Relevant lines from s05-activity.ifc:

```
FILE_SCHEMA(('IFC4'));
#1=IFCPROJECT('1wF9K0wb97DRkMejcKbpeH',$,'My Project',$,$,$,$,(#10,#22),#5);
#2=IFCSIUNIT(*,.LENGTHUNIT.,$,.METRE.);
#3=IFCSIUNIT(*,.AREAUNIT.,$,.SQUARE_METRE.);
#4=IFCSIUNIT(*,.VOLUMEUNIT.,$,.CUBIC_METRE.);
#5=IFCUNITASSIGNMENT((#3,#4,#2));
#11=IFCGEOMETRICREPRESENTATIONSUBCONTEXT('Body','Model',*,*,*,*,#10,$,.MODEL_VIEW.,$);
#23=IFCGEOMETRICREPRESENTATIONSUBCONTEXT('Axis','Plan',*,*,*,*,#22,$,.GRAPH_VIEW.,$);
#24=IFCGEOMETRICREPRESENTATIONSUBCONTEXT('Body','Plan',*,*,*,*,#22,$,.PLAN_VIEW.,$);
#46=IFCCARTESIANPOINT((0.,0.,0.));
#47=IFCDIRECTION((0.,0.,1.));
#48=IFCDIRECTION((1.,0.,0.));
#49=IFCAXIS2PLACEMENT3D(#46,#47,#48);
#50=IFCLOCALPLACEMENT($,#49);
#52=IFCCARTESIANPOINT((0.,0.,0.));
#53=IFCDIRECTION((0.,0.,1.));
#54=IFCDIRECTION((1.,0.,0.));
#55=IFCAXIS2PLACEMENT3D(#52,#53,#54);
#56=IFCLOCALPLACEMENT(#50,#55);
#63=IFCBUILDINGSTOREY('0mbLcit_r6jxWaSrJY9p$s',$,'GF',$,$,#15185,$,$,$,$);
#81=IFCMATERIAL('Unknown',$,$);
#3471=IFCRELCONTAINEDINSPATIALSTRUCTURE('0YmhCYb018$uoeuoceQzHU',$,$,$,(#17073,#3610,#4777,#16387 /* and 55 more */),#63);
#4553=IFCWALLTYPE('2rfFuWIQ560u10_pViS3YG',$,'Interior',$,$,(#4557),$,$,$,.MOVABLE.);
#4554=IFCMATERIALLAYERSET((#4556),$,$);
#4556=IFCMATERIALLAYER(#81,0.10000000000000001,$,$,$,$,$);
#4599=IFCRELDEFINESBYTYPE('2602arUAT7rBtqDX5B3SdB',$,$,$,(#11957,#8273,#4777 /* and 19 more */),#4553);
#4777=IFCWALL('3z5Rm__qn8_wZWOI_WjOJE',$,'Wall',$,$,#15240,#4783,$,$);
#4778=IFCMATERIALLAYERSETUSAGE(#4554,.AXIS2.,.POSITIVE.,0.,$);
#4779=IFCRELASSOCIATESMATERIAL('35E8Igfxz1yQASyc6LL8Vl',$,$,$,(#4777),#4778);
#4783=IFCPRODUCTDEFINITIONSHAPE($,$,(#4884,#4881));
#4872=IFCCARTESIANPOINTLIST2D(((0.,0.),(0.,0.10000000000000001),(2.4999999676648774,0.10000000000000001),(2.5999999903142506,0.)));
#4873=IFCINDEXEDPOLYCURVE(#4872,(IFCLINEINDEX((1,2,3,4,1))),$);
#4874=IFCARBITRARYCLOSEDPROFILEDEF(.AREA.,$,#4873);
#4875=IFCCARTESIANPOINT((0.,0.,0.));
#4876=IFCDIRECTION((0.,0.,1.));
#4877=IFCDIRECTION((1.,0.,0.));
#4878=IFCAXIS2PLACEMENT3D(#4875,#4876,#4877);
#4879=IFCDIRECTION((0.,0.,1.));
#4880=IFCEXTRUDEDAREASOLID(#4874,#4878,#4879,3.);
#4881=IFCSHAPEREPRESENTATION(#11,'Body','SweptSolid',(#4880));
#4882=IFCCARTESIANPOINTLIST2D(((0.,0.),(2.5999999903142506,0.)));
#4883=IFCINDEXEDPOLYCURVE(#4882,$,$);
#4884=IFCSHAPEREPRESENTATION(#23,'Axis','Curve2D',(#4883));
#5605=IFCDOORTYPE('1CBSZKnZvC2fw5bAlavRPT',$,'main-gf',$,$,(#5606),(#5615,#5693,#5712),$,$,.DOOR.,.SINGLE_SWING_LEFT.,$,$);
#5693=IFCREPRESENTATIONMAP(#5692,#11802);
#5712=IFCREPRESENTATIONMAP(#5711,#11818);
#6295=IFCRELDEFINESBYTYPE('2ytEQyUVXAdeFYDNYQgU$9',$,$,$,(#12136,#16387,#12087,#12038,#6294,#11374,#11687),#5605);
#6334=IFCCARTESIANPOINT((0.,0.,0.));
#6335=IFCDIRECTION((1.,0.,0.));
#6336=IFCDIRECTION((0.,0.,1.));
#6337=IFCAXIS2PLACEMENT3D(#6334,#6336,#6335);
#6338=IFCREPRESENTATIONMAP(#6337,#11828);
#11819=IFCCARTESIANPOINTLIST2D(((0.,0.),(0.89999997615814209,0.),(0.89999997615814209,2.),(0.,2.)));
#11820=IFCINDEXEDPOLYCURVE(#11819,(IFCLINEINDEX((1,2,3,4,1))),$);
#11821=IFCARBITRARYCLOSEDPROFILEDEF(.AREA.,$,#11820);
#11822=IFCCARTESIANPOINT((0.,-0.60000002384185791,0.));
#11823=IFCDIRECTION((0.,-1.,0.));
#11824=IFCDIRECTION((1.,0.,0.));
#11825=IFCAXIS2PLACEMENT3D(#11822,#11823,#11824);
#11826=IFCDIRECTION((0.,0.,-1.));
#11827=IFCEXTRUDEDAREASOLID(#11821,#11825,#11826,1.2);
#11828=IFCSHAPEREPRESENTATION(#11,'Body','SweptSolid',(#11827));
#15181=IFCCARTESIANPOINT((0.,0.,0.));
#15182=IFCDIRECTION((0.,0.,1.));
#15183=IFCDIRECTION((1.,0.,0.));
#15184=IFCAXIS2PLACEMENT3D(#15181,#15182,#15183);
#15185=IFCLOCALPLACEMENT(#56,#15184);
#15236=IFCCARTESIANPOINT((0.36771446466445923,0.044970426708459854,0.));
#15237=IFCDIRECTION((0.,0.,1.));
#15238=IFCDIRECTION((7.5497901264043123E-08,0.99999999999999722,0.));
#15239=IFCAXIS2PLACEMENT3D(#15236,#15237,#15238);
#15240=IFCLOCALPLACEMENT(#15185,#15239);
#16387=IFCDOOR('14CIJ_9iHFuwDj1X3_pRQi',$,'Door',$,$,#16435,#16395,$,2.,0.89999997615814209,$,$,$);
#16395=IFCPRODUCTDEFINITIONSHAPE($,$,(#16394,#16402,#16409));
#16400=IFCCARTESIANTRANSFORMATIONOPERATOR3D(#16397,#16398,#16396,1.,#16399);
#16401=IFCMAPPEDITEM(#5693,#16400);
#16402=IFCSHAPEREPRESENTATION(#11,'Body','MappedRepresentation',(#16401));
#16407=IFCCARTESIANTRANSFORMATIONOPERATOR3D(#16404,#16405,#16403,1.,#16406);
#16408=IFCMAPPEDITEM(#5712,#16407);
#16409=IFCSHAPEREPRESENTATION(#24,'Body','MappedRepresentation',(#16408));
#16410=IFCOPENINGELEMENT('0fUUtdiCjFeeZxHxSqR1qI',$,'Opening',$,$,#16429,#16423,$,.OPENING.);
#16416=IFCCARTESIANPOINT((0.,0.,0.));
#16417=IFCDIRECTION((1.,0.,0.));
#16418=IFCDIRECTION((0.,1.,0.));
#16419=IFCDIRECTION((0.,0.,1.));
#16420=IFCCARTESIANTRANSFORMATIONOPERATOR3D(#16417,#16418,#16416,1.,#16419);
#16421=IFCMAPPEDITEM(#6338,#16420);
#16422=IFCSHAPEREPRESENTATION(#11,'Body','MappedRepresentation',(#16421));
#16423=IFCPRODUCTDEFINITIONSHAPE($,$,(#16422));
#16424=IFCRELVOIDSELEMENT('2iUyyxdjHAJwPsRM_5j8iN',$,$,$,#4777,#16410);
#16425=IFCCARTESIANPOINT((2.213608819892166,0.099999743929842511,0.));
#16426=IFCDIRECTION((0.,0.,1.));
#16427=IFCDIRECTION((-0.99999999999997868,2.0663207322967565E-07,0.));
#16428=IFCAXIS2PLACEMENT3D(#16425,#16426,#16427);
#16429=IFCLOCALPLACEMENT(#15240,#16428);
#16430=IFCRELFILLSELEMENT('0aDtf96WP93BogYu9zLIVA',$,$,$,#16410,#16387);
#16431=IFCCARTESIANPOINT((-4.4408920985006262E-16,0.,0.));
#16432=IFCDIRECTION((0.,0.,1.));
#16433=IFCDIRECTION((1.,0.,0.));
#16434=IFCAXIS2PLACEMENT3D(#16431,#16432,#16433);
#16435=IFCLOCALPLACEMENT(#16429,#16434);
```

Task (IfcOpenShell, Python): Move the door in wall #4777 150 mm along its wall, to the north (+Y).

```python
import ifcopenshell
import ifcopenshell.api.geometry
import ifcopenshell.util.placement
import ifcopenshell.util.unit

model = ifcopenshell.open("s05-activity.ifc")
unit_scale = ifcopenshell.util.unit.calculate_unit_scale(model)

door = model.by_id(16387)
opening = door.FillsVoids[0].RelatingOpeningElement
wall = opening.VoidsElements[0].RelatingBuildingElement

wall_matrix = ifcopenshell.util.placement.get_local_placement(wall.ObjectPlacement)
shift = wall_matrix[:3, 0] * 0.15 / unit_scale
before = ifcopenshell.util.placement.get_local_placement(door.ObjectPlacement)[:3, 3].copy()

# The door is placed relative to its opening, so it follows when the opening moves.
matrix = ifcopenshell.util.placement.get_local_placement(opening.ObjectPlacement)
matrix[:3, 3] += shift
ifcopenshell.api.geometry.edit_object_placement(
    model, product=opening, matrix=matrix, is_si=False, should_transform_children=True
)

after = ifcopenshell.util.placement.get_local_placement(door.ObjectPlacement)[:3, 3]
print("door moved by", (after - before).round(3) + 0.0)

model.write("s05-activity_edited.ifc")
```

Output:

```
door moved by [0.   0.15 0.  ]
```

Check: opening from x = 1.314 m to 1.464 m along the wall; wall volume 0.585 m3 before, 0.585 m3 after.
